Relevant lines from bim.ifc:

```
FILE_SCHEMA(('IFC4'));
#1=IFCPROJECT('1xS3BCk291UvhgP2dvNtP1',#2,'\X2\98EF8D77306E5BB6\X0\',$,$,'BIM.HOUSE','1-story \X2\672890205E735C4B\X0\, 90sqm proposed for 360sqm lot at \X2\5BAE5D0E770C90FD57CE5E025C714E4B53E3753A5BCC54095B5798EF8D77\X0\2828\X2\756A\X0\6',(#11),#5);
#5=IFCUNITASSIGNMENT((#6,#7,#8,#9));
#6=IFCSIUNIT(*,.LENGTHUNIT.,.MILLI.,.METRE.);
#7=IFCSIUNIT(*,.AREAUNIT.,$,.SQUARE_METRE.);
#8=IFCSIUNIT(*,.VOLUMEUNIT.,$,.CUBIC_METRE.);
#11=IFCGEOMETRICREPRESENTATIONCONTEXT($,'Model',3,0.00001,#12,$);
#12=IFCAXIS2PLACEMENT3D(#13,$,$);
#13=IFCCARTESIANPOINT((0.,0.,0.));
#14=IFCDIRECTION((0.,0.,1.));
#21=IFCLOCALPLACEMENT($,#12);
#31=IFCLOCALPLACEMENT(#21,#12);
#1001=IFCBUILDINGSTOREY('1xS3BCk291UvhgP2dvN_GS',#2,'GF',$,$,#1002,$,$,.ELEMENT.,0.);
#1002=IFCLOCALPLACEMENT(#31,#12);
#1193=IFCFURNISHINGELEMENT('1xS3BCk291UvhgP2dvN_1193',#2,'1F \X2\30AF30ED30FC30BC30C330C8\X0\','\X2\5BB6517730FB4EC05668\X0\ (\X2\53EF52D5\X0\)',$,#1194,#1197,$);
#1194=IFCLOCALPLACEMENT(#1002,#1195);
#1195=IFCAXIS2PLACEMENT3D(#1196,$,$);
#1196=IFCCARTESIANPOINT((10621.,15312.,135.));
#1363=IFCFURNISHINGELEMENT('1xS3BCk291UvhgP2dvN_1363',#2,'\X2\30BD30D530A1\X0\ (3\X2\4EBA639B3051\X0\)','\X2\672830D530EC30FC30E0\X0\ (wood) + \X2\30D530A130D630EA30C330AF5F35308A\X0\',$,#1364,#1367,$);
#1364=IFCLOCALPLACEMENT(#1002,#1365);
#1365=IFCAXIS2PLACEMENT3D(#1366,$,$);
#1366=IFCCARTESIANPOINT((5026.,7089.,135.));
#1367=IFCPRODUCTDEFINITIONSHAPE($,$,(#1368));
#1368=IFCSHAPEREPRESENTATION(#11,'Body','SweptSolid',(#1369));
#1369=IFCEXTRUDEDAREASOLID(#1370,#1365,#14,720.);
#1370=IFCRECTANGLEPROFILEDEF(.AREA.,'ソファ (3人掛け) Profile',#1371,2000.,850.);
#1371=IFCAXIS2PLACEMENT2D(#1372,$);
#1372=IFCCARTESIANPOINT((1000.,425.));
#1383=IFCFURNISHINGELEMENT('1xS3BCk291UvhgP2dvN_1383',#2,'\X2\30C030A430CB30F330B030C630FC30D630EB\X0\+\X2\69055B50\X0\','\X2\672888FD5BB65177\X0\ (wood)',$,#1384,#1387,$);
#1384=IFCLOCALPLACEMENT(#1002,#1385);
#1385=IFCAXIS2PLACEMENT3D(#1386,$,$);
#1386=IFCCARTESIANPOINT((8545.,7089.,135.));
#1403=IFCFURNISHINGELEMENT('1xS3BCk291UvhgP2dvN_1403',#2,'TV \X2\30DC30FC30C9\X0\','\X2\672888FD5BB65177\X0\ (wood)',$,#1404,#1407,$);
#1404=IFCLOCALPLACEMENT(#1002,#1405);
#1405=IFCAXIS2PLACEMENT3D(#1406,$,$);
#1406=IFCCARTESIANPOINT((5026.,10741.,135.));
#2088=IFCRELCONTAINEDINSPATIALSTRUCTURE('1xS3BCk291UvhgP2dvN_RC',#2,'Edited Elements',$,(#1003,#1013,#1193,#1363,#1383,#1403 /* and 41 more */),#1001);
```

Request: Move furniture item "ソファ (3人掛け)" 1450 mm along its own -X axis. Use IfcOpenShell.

```python
import ifcopenshell
import ifcopenshell.api.geometry
import ifcopenshell.util.placement
import ifcopenshell.util.unit

model = ifcopenshell.open("bim.ifc")
unit_scale = ifcopenshell.util.unit.calculate_unit_scale(model)

item = model.by_guid("1xS3BCk291UvhgP2dvN_1363")
matrix = ifcopenshell.util.placement.get_local_placement(item.ObjectPlacement)
matrix[:3, 3] -= matrix[:3, 0] * 1.45 / unit_scale
ifcopenshell.api.geometry.edit_object_placement(model, product=item, matrix=matrix, is_si=False)

print(ifcopenshell.util.placement.get_local_placement(item.ObjectPlacement).round(3) + 0.0)

model.write("bim_rev.ifc")
```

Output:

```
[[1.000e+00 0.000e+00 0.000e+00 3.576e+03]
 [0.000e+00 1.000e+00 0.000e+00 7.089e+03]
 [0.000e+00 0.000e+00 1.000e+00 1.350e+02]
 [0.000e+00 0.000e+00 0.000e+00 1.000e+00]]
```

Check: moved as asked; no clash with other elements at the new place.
